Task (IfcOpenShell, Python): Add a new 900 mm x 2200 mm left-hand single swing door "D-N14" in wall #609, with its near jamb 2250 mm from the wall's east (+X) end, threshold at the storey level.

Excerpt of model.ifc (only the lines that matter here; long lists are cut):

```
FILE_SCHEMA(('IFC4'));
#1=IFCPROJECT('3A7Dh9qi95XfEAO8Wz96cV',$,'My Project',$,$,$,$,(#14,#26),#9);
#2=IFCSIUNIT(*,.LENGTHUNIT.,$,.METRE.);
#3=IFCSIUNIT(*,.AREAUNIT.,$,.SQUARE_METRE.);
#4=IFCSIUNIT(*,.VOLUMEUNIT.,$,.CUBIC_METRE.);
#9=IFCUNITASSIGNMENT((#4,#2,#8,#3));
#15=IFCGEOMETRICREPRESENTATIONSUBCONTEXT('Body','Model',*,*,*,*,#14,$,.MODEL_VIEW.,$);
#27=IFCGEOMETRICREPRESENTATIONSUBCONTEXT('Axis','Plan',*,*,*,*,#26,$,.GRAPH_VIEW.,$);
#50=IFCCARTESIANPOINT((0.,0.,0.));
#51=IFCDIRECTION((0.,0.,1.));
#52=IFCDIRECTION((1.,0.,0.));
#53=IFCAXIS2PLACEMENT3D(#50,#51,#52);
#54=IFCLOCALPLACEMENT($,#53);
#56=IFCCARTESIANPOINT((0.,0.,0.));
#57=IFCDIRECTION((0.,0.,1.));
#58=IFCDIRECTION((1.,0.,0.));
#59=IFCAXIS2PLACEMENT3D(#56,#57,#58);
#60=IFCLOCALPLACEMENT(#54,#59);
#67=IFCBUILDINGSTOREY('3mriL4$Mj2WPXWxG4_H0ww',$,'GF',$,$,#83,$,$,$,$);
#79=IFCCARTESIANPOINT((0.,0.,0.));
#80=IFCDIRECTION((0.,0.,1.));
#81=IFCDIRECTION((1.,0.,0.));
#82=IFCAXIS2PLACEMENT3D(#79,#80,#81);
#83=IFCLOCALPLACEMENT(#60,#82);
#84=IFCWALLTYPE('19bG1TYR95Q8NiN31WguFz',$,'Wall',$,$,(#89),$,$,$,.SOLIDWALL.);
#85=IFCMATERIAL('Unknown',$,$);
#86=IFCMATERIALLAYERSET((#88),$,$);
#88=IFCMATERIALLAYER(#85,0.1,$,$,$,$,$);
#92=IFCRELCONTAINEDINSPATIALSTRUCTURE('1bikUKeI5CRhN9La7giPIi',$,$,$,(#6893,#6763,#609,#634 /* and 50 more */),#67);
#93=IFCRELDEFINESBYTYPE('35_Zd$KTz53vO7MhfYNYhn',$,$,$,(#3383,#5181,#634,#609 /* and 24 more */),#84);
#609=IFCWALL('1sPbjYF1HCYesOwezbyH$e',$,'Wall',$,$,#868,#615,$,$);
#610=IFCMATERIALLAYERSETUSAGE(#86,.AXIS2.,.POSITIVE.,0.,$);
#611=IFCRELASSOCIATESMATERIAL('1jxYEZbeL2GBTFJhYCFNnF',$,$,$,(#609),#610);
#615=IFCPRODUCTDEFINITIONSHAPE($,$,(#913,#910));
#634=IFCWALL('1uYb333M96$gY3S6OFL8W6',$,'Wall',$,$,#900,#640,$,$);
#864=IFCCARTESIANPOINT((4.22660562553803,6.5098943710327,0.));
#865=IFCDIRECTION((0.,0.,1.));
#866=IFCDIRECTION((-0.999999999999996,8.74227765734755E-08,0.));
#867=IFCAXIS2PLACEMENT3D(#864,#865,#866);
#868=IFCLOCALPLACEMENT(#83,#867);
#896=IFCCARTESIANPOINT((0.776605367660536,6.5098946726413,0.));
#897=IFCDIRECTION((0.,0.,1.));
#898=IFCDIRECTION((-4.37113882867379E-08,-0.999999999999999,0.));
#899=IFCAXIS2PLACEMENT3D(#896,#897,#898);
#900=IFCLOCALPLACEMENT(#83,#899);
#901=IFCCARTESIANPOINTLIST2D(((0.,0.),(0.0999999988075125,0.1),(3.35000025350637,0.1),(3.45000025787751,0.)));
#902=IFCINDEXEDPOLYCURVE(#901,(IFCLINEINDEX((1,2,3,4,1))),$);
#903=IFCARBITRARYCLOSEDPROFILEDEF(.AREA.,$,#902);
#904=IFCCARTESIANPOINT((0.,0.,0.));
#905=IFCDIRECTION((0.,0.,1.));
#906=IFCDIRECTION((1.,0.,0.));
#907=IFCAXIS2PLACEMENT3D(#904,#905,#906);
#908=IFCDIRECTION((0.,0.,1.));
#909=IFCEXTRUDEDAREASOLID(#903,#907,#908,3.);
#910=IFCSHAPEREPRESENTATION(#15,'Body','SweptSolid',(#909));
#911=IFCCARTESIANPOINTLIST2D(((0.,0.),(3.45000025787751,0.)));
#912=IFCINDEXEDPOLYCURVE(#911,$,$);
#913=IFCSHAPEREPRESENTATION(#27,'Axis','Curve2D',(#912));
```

```python
import numpy as np
import ifcopenshell
import ifcopenshell.api.feature
import ifcopenshell.api.geometry
import ifcopenshell.api.root
import ifcopenshell.api.spatial
import ifcopenshell.geom
import ifcopenshell.util.element
import ifcopenshell.util.placement
import ifcopenshell.util.representation
import ifcopenshell.util.shape
import ifcopenshell.util.unit

model = ifcopenshell.open("model.ifc")
unit_scale = ifcopenshell.util.unit.calculate_unit_scale(model)
settings = ifcopenshell.geom.settings()


def volume(element):
    """Net volume in cubic metres, openings subtracted."""
    shape = ifcopenshell.geom.create_shape(settings, element)
    return ifcopenshell.util.shape.get_volume(shape.geometry)


wall = model.by_id(609)
storey = ifcopenshell.util.element.get_container(wall, ifc_class="IfcBuildingStorey")
context = ifcopenshell.util.representation.get_context(model, "Model", "Body", "MODEL_VIEW")
before = volume(wall)

width, height, from_end, sill = 0.9, 2.2, 2.25, 0.0  # metres

# The wall runs along its own X axis, and the end named is its -X end.
wall_shape = ifcopenshell.geom.create_shape(settings, wall)
x, y, z = ifcopenshell.util.shape.get_vertices(wall_shape.geometry).T
start = x.min() + from_end
face, thickness = float(y.min()), float(y.max() - y.min())
wall_matrix = ifcopenshell.util.placement.get_local_placement(wall.ObjectPlacement)
level = ifcopenshell.util.placement.get_local_placement(storey.ObjectPlacement)[2, 3]


def in_wall(x, y):
    """Placement at x, y metres in the wall's axes, at sill height."""
    matrix = wall_matrix.copy()
    matrix[:, 3] = wall_matrix @ np.array([x / unit_scale, y / unit_scale, 0.0, 1.0])
    matrix[2, 3] = level + sill / unit_scale
    return matrix


# Opening: a box that overshoots both wall faces by 50 mm.
opening = ifcopenshell.api.root.create_entity(model, ifc_class="IfcOpeningElement", predefined_type="OPENING")
box = ifcopenshell.api.geometry.add_wall_representation(
    model, context=context, length=width, height=height, thickness=thickness + 0.1
)
ifcopenshell.api.geometry.assign_representation(model, product=opening, representation=box)
ifcopenshell.api.geometry.edit_object_placement(model, product=opening, matrix=in_wall(start, face - 0.05), is_si=False)
ifcopenshell.api.feature.add_feature(model, feature=opening, element=wall)

door = ifcopenshell.api.root.create_entity(model, ifc_class="IfcDoor", name="D-N14", predefined_type="DOOR")
door.OverallWidth, door.OverallHeight = width / unit_scale, height / unit_scale
door.OperationType = "SINGLE_SWING_LEFT"
body = ifcopenshell.api.geometry.add_door_representation(
    model,
    context=context,
    overall_width=door.OverallWidth,
    overall_height=door.OverallHeight,
    operation_type="SINGLE_SWING_LEFT",
    lining_properties={"LiningDepth": thickness / unit_scale, "ThresholdDepth": thickness / unit_scale},
)
ifcopenshell.api.geometry.assign_representation(model, product=door, representation=body)
ifcopenshell.api.spatial.assign_container(model, products=[door], relating_structure=storey)
ifcopenshell.api.feature.add_filling(model, opening=opening, element=door)

# The lining spans the wall, so the door starts at the wall face.
ifcopenshell.api.geometry.edit_object_placement(model, product=door, matrix=in_wall(start, face), is_si=False)

after = volume(wall)

print(f"wall volume {before:.3f} -> {after:.3f} m3")

model.write("model-out.ifc")
```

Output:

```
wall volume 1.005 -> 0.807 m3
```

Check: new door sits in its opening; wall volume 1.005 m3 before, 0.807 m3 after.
